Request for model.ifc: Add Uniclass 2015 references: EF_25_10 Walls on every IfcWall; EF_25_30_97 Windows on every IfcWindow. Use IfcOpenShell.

First a look at what the model holds.

```python
import ifcopenshell

model = ifcopenshell.open("model.ifc")
print(model.schema)
print("classifications:", [c.Name for c in model.by_type("IfcClassification")])
for ifc_class in ("IfcDoor", "IfcRoof", "IfcStair", "IfcWall", "IfcWindow"):
    print(ifc_class, len(model.by_type(ifc_class)))
```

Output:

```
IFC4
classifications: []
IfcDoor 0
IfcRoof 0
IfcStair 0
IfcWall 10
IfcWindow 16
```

```python
import ifcopenshell
import ifcopenshell.api.classification

model = ifcopenshell.open("model.ifc")

system = ifcopenshell.api.classification.add_classification(model, classification="Uniclass 2015")

codes = {
    "IfcWall": ("EF_25_10", "Walls"),
    "IfcWindow": ("EF_25_30_97", "Windows"),
}
for ifc_class, (code, name) in codes.items():
    products = model.by_type(ifc_class)
    ifcopenshell.api.classification.add_reference(
        model, products=products, classification=system, identification=code, name=name
    )
    print(code, len(products))

model.write("model_edited.ifc")
```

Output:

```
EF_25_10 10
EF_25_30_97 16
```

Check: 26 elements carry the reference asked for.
